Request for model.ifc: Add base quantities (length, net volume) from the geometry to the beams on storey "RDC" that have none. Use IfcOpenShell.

First a look at what the model holds.

```python
import ifcopenshell
import ifcopenshell.util.element
import ifcopenshell.util.unit

model = ifcopenshell.open("model.ifc")
print(model.schema)
for unit_type in ("LENGTHUNIT", "AREAUNIT", "VOLUMEUNIT"):
    print(unit_type, ifcopenshell.util.unit.calculate_unit_scale(model, unit_type))
storey = next(s for s in model.by_type("IfcBuildingStorey") if s.Name == "RDC")
beams = [e for e in ifcopenshell.util.element.get_decomposition(storey) if e.is_a("IfcBeam")]
for e in sorted(beams, key=lambda e: e.id()):
    print(e.id(), e.is_a(), e.Name, list(ifcopenshell.util.element.get_psets(e, qtos_only=True)), sep=" | ")
```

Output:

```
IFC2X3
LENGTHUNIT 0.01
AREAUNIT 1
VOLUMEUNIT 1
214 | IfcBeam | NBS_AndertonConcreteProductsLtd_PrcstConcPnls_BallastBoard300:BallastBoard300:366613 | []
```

```python
import ifcopenshell
import ifcopenshell.api.pset
import ifcopenshell.geom
import ifcopenshell.util.element
import ifcopenshell.util.shape
import ifcopenshell.util.unit

model = ifcopenshell.open("model.ifc")
unit_scale = ifcopenshell.util.unit.calculate_unit_scale(model)
volume_scale = ifcopenshell.util.unit.calculate_unit_scale(model, "VOLUMEUNIT")
settings = ifcopenshell.geom.settings()

storey = next(s for s in model.by_type("IfcBuildingStorey") if s.Name == "RDC")
beams = [e for e in ifcopenshell.util.element.get_decomposition(storey) if e.is_a("IfcBeam")]

for e in sorted(beams, key=lambda e: e.id()):
    if ifcopenshell.util.element.get_psets(e, qtos_only=True, should_inherit=False):
        continue
    # Geometry comes back in metres, in the element's own axes.
    shape = ifcopenshell.geom.create_shape(settings, e)
    values = {
        "Length": ifcopenshell.util.shape.get_max_xyz(shape.geometry) / unit_scale,
        "NetVolume": ifcopenshell.util.shape.get_volume(shape.geometry) / volume_scale,
    }
    qto = ifcopenshell.api.pset.add_qto(model, product=e, name="BaseQuantities")
    ifcopenshell.api.pset.edit_qto(model, qto=qto, properties=values)
    print(e.id(), {k: round(v, 3) for k, v in values.items()})

model.write("model_edited.ifc")
```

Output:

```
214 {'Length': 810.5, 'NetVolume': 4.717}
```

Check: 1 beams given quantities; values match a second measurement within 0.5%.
